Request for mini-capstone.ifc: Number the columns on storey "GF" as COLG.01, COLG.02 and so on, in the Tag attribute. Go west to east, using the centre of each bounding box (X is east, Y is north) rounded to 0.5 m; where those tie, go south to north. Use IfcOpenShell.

First a look at what the model holds.

```python
import ifcopenshell
import ifcopenshell.util.element
import ifcopenshell.util.placement

model = ifcopenshell.open("mini-capstone.ifc")
print(model.schema)
storey = next(s for s in model.by_type("IfcBuildingStorey") if s.Name == "GF")
columns = [e for e in ifcopenshell.util.element.get_decomposition(storey) if e.is_a("IfcColumn")]
for e in sorted(columns, key=lambda e: e.id()):
    origin = ifcopenshell.util.placement.get_local_placement(e.ObjectPlacement)[:3, 3]
    print(e.id(), e.Tag, e.Name, origin.round(2) + 0.0, sep=" | ")
```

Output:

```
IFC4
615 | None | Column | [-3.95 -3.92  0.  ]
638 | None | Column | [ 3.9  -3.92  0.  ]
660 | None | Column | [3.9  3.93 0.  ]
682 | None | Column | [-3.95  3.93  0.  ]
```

```python
import ifcopenshell
import ifcopenshell.geom
import ifcopenshell.util.element
import ifcopenshell.util.shape

model = ifcopenshell.open("mini-capstone.ifc")
settings = ifcopenshell.geom.settings()
settings.set("use-world-coords", True)


def centre(element):
    shape = ifcopenshell.geom.create_shape(settings, element)
    return ifcopenshell.util.shape.get_bbox_centroid(shape.geometry)


storey = next(s for s in model.by_type("IfcBuildingStorey") if s.Name == "GF")
columns = [e for e in ifcopenshell.util.element.get_decomposition(storey) if e.is_a("IfcColumn")]

# Insertion points can sit at a corner or the storey origin, so sort by the geometry (in metres).
centres = {e: centre(e) for e in columns}
columns.sort(key=lambda e: (round(centres[e][0] / 0.5), centres[e][1]))

for i, e in enumerate(columns, start=1):
    number = f"COLG.{i:02d}"
    e.Tag = number
    print(e.id(), number)

model.write("mini-capstone_v2.ifc")
```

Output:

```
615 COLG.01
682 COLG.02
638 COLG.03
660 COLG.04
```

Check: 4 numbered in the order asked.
